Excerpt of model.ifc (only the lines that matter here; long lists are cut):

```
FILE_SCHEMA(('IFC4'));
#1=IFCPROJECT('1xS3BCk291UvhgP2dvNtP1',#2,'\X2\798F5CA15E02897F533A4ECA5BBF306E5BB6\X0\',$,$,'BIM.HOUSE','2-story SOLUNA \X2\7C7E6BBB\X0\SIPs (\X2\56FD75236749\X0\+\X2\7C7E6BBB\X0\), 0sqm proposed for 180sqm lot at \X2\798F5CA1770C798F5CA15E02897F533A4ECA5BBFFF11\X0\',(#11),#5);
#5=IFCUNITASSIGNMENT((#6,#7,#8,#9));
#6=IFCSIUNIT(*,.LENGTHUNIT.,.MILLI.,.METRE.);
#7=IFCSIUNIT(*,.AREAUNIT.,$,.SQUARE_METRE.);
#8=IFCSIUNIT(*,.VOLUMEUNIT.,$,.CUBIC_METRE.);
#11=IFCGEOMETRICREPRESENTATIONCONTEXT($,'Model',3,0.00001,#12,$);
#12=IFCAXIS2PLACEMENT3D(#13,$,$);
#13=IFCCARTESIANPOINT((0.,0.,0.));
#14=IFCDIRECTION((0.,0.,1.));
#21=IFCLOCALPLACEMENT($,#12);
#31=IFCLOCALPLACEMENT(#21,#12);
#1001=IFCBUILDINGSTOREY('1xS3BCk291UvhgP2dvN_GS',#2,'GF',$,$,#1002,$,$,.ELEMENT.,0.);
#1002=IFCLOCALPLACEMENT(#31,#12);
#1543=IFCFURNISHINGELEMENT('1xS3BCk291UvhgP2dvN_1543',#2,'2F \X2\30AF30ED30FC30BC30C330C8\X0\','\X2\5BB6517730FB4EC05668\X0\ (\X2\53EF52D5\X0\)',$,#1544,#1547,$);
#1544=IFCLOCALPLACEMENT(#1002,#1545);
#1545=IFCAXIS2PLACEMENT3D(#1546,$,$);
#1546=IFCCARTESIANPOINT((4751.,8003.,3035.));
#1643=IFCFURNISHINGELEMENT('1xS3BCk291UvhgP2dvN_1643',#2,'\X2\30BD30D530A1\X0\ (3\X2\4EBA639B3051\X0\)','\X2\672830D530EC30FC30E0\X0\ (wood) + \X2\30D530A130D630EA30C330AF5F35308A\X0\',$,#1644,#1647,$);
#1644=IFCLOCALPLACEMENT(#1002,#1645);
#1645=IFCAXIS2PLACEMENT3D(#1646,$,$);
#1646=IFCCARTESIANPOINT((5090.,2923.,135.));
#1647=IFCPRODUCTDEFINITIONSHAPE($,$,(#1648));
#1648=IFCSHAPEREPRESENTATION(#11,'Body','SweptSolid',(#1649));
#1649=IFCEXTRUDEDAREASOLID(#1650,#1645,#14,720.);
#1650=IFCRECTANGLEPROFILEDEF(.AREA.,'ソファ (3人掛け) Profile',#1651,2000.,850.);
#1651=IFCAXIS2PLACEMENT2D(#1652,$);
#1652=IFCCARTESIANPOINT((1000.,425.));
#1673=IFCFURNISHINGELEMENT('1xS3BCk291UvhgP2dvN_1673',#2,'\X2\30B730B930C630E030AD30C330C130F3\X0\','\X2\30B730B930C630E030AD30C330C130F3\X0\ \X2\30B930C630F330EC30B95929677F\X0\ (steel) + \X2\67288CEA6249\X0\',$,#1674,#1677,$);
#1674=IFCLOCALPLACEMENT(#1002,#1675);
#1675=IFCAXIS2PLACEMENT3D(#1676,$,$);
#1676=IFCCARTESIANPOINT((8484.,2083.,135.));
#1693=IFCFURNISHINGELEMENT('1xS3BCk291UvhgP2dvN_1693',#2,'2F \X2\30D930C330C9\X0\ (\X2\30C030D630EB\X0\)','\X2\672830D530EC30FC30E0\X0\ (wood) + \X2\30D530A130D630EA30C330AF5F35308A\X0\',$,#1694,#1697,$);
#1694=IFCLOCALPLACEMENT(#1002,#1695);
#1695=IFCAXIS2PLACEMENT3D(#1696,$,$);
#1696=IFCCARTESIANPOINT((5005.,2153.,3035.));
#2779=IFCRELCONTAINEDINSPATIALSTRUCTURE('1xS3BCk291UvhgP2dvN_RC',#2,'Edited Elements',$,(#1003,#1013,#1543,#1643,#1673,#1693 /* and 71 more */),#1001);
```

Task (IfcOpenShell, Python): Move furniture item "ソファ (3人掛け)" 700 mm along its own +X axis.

```python
import ifcopenshell
import ifcopenshell.api.geometry
import ifcopenshell.util.placement
import ifcopenshell.util.unit

model = ifcopenshell.open("model.ifc")
unit_scale = ifcopenshell.util.unit.calculate_unit_scale(model)

item = model.by_id(1643)
matrix = ifcopenshell.util.placement.get_local_placement(item.ObjectPlacement)
matrix[:3, 3] += matrix[:3, 0] * 0.7 / unit_scale
ifcopenshell.api.geometry.edit_object_placement(model, product=item, matrix=matrix, is_si=False)

print(ifcopenshell.util.placement.get_local_placement(item.ObjectPlacement).round(3) + 0.0)

model.write("model_edited.ifc")
```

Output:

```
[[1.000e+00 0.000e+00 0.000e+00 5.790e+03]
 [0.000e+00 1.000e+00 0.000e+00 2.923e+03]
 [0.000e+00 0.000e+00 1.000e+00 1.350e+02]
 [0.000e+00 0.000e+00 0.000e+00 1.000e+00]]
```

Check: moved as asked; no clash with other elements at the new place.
